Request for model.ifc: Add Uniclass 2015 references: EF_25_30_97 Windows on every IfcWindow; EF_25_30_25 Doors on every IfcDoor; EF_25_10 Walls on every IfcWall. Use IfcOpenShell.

First a look at what the model holds.

```python
import ifcopenshell

model = ifcopenshell.open("model.ifc")
print(model.schema)
print("classifications:", [c.Name for c in model.by_type("IfcClassification")])
for ifc_class in ("IfcDoor", "IfcRoof", "IfcStair", "IfcWall", "IfcWindow"):
    print(ifc_class, len(model.by_type(ifc_class)))
```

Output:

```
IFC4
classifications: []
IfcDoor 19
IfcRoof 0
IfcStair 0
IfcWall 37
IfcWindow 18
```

```python
import ifcopenshell
import ifcopenshell.api.classification

model = ifcopenshell.open("model.ifc")

system = ifcopenshell.api.classification.add_classification(model, classification="Uniclass 2015")

codes = {
    "IfcWindow": ("EF_25_30_97", "Windows"),
    "IfcDoor": ("EF_25_30_25", "Doors"),
    "IfcWall": ("EF_25_10", "Walls"),
}
for ifc_class, (code, name) in codes.items():
    products = model.by_type(ifc_class)
    ifcopenshell.api.classification.add_reference(
        model, products=products, classification=system, identification=code, name=name
    )
    print(code, len(products))

model.write("model_rev.ifc")
```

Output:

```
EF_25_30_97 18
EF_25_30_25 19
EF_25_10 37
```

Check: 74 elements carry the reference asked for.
